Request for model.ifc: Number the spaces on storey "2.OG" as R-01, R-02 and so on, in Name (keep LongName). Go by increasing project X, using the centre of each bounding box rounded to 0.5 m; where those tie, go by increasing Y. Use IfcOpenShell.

First a look at what the model holds.

```python
import ifcopenshell
import ifcopenshell.util.element
import ifcopenshell.util.placement

model = ifcopenshell.open("model.ifc")
print(model.schema)
storey = next(s for s in model.by_type("IfcBuildingStorey") if s.Name == "2.OG")
spaces = [e for e in ifcopenshell.util.element.get_decomposition(storey) if e.is_a("IfcSpace")]
for e in sorted(spaces, key=lambda e: e.id()):
    origin = ifcopenshell.util.placement.get_local_placement(e.ObjectPlacement)[:3, 3]
    print(e.id(), e.Name, e.LongName, origin.round(2) + 0.0, sep=" | ")
```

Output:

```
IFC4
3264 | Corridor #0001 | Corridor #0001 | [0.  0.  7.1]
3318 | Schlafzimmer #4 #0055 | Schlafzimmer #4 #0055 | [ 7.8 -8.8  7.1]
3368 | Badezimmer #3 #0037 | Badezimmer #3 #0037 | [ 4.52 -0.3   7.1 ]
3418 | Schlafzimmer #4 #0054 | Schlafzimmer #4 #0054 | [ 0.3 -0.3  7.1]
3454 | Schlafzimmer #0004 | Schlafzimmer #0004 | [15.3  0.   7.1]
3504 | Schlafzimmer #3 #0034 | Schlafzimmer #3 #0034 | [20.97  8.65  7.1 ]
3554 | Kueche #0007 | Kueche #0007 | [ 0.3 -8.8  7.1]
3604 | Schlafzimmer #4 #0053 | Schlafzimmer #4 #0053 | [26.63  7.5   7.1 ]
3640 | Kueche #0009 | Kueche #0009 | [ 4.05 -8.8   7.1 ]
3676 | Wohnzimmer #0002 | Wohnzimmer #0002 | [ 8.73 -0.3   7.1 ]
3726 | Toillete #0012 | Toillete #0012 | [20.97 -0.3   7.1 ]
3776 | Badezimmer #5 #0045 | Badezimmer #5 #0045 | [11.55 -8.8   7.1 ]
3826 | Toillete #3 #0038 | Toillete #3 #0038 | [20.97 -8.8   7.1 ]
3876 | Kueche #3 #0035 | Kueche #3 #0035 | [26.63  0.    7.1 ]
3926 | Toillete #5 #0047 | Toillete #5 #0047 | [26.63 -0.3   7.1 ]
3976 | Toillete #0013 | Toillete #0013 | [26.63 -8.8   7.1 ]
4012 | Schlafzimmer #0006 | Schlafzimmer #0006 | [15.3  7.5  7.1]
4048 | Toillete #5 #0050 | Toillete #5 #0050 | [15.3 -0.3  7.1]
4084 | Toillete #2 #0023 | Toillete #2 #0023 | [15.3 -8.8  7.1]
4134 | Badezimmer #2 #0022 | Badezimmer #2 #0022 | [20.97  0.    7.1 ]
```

```python
import ifcopenshell
import ifcopenshell.geom
import ifcopenshell.util.element
import ifcopenshell.util.shape

model = ifcopenshell.open("model.ifc")
settings = ifcopenshell.geom.settings()
settings.set("use-world-coords", True)


def centre(element):
    shape = ifcopenshell.geom.create_shape(settings, element)
    return ifcopenshell.util.shape.get_bbox_centroid(shape.geometry)


storey = next(s for s in model.by_type("IfcBuildingStorey") if s.Name == "2.OG")
spaces = [e for e in ifcopenshell.util.element.get_decomposition(storey) if e.is_a("IfcSpace")]

# Insertion points can sit at a corner or the storey origin, so sort by the geometry (in metres).
centres = {e: centre(e) for e in spaces}
spaces.sort(key=lambda e: (round(centres[e][0] / 0.5), centres[e][1]))

for i, e in enumerate(spaces, start=1):
    number = f"R-{i:02d}"
    e.Name = number
    print(e.id(), number)

model.write("model_updated.ifc")
```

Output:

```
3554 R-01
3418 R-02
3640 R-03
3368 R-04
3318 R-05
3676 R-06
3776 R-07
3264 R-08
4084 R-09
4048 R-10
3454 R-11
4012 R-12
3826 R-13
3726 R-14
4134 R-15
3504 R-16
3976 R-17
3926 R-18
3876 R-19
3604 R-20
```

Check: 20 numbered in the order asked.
